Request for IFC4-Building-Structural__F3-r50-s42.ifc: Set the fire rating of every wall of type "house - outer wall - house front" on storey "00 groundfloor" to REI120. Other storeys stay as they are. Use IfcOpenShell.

First a look at what the model holds.

```python
import ifcopenshell
import ifcopenshell.util.element

model = ifcopenshell.open("IFC4-Building-Structural__F3-r50-s42.ifc")
print(model.schema)
storey = next(s for s in model.by_type("IfcBuildingStorey") if s.Name == "00 groundfloor")
walls = [e for e in ifcopenshell.util.element.get_decomposition(storey) if e.is_a("IfcWall")]
seen = {}
for e in walls:
    element_type = ifcopenshell.util.element.get_type(e)
    key = (element_type.Name if element_type != e and element_type else None, ifcopenshell.util.element.get_pset(e, "Pset_WallCommon", "FireRating"))
    seen[key] = seen.get(key, 0) + 1
for (name, value), count in sorted(seen.items(), key=str):
    print(count, "x", name, "|", value)
```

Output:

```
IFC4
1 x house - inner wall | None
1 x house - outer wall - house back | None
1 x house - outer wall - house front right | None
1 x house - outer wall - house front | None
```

```python
import ifcopenshell
import ifcopenshell.api.pset
import ifcopenshell.util.element

model = ifcopenshell.open("IFC4-Building-Structural__F3-r50-s42.ifc")

storey = next(s for s in model.by_type("IfcBuildingStorey") if s.Name == "00 groundfloor")
walls = [e for e in ifcopenshell.util.element.get_decomposition(storey) if e.is_a("IfcWall")]

count = 0
for e in walls:
    element_type = ifcopenshell.util.element.get_type(e)
    if element_type in (None, e) or element_type.Name != "house - outer wall - house front":
        continue
    # add_pset returns the element's existing set when there is one.
    pset = ifcopenshell.api.pset.add_pset(model, product=e, name="Pset_WallCommon")
    ifcopenshell.api.pset.edit_pset(model, pset=pset, properties={"FireRating": "REI120"})
    count += 1

print(count, "walls updated")

model.write("IFC4-Building-Structural__F3-r50-s42_edited.ifc")
```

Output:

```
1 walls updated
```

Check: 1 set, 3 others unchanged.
